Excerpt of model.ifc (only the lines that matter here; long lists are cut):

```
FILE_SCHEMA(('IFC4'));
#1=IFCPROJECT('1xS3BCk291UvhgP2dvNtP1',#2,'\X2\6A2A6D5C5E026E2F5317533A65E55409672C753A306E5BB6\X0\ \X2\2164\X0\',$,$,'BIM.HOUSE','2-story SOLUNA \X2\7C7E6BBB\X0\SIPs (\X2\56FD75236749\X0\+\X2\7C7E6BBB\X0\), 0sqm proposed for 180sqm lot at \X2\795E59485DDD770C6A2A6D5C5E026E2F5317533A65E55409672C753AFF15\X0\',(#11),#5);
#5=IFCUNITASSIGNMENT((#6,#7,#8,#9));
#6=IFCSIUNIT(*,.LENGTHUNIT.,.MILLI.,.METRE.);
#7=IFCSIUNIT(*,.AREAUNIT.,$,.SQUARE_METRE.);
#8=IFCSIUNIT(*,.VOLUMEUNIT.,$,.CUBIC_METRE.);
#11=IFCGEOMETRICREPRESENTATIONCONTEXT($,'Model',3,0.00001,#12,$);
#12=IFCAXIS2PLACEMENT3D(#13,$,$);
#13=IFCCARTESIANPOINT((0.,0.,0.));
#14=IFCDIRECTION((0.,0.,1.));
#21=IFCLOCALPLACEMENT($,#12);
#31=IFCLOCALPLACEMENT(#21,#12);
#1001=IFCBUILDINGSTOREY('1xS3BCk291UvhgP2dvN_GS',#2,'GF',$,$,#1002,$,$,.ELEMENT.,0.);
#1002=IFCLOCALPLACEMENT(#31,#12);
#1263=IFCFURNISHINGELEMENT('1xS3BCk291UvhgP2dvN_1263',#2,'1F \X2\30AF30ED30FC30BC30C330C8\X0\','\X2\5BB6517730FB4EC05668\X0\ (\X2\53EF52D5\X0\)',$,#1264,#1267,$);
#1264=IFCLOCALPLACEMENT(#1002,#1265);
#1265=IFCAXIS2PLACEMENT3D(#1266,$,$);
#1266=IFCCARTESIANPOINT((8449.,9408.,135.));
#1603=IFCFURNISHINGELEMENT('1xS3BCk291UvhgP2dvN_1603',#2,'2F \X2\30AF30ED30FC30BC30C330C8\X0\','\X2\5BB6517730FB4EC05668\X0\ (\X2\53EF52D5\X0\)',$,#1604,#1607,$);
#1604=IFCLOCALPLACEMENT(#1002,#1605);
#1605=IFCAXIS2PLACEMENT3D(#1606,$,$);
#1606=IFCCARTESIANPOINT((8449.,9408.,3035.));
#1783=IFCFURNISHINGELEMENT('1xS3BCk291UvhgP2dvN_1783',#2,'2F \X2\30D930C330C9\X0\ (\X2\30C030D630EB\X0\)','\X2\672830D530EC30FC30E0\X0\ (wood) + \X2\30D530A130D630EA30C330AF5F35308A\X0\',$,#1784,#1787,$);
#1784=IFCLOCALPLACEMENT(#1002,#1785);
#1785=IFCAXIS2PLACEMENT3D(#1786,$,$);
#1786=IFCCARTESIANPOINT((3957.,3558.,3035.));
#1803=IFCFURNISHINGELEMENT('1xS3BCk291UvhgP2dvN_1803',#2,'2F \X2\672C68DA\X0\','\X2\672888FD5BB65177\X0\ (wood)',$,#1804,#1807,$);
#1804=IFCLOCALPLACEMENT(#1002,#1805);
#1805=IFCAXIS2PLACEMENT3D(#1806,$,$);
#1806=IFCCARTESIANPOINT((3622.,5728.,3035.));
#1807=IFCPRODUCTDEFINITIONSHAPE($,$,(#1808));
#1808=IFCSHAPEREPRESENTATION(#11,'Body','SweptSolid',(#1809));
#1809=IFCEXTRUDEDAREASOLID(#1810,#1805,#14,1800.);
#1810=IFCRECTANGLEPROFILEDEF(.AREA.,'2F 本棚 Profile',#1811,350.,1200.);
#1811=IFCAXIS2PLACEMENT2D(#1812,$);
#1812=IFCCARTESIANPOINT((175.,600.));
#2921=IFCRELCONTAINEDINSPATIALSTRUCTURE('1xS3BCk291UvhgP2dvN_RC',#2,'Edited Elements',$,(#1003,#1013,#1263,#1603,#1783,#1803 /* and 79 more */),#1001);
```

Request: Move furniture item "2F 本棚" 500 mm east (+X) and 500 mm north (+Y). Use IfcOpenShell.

```python
import ifcopenshell
import ifcopenshell.api.geometry
import ifcopenshell.util.placement
import ifcopenshell.util.unit

model = ifcopenshell.open("model.ifc")
unit_scale = ifcopenshell.util.unit.calculate_unit_scale(model)

item = model.by_guid("1xS3BCk291UvhgP2dvN_1803")
matrix = ifcopenshell.util.placement.get_local_placement(item.ObjectPlacement)
matrix[0, 3] += 0.5 / unit_scale
matrix[1, 3] += 0.5 / unit_scale
ifcopenshell.api.geometry.edit_object_placement(model, product=item, matrix=matrix, is_si=False)

print(ifcopenshell.util.placement.get_local_placement(item.ObjectPlacement).round(3) + 0.0)

model.write("model_rev.ifc")
```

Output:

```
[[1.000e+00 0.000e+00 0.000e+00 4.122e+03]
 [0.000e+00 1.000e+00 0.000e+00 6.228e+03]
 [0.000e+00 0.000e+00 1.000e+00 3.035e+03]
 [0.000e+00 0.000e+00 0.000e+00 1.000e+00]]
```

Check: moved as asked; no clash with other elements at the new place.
